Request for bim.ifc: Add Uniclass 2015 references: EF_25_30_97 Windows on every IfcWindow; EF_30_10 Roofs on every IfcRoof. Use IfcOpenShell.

First a look at what the model holds.

```python
import ifcopenshell

model = ifcopenshell.open("bim.ifc")
print(model.schema)
print("classifications:", [c.Name for c in model.by_type("IfcClassification")])
for ifc_class in ("IfcDoor", "IfcRoof", "IfcStair", "IfcWall", "IfcWindow"):
    print(ifc_class, len(model.by_type(ifc_class)))
```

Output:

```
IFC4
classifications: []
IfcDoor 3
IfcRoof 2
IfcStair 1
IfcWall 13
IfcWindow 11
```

```python
import ifcopenshell
import ifcopenshell.api.classification

model = ifcopenshell.open("bim.ifc")

system = ifcopenshell.api.classification.add_classification(model, classification="Uniclass 2015")

codes = {
    "IfcWindow": ("EF_25_30_97", "Windows"),
    "IfcRoof": ("EF_30_10", "Roofs"),
}
for ifc_class, (code, name) in codes.items():
    products = model.by_type(ifc_class)
    ifcopenshell.api.classification.add_reference(
        model, products=products, classification=system, identification=code, name=name
    )
    print(code, len(products))

model.write("bim_edited.ifc")
```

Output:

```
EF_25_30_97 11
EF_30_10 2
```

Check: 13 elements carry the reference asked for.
